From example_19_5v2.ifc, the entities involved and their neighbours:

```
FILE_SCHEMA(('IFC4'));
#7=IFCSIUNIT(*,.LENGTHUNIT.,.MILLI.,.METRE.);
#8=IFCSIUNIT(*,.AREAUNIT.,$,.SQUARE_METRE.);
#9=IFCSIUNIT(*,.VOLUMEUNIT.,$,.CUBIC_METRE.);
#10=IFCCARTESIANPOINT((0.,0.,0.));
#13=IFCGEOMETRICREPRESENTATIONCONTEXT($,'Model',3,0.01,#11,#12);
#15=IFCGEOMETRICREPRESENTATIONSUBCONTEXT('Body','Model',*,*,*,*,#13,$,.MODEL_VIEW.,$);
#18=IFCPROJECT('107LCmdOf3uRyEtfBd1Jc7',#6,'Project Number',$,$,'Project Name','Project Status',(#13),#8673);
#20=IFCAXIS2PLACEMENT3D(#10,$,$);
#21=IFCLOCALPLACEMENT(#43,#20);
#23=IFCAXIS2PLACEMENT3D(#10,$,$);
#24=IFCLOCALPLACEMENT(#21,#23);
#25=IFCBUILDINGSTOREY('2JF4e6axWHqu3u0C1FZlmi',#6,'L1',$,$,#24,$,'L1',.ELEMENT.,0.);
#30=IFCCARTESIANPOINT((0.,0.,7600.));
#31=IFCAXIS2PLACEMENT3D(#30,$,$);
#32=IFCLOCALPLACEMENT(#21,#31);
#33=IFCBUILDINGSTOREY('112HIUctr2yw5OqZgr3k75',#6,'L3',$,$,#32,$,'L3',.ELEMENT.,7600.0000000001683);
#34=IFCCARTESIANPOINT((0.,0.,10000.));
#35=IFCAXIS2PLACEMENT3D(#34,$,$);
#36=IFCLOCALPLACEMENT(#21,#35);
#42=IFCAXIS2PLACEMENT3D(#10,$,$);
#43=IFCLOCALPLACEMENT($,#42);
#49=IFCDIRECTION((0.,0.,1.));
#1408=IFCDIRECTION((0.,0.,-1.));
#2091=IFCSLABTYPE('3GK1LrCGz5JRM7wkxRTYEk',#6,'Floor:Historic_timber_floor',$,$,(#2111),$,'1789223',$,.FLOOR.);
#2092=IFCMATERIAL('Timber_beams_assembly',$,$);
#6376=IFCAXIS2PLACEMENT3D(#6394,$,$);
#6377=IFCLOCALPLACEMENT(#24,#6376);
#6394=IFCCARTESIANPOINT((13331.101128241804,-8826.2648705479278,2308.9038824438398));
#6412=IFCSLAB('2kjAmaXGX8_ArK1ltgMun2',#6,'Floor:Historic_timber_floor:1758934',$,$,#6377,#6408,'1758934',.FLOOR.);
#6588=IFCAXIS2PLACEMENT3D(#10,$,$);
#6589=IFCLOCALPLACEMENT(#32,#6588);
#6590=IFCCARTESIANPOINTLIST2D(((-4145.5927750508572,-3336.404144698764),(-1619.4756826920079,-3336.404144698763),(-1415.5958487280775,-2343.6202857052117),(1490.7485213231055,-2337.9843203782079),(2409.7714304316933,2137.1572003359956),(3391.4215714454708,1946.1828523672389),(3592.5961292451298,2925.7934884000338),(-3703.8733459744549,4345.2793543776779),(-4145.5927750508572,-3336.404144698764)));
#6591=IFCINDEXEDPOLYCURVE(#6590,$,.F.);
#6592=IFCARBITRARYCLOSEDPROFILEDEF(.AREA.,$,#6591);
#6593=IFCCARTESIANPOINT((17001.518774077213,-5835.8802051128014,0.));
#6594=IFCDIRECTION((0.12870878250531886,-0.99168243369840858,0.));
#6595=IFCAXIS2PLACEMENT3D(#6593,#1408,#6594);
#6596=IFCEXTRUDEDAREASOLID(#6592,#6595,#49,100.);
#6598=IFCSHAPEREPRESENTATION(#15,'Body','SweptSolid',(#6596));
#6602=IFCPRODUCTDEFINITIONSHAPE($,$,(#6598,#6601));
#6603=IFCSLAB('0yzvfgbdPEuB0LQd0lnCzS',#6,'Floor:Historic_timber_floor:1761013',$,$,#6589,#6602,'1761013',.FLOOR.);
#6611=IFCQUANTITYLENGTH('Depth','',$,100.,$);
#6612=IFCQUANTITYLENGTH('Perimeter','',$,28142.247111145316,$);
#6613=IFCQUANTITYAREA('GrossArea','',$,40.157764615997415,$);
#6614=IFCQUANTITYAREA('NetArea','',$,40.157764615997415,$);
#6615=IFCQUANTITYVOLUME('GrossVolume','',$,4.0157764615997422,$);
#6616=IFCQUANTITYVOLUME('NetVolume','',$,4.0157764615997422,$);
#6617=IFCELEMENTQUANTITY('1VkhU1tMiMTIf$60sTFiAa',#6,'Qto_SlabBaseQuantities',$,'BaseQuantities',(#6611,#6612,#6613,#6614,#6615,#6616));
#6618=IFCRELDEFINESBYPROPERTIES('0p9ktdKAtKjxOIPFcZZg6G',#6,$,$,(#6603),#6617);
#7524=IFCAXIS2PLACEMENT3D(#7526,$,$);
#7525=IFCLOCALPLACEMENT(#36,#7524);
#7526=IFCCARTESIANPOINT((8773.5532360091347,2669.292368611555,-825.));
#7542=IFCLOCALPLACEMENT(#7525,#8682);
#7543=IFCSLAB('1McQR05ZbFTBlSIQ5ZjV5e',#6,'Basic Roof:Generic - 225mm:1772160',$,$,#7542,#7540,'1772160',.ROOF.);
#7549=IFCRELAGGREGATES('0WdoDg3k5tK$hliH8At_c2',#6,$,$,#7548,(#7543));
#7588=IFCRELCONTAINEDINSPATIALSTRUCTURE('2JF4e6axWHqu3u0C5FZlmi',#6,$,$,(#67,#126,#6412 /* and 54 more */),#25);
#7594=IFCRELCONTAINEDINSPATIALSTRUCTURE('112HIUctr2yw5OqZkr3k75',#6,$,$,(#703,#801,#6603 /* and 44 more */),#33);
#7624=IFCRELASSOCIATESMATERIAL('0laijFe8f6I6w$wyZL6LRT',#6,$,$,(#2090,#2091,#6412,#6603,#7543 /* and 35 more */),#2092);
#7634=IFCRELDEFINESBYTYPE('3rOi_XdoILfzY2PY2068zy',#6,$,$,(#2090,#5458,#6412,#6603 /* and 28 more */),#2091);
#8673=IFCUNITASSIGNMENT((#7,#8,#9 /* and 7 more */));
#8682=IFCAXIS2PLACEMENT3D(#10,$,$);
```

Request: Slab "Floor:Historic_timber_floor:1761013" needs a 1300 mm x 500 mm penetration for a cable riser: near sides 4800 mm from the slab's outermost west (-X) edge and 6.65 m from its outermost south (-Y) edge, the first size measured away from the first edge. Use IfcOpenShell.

```python
import numpy as np
import ifcopenshell
import ifcopenshell.api.feature
import ifcopenshell.api.geometry
import ifcopenshell.api.pset
import ifcopenshell.api.root
import ifcopenshell.geom
import ifcopenshell.util.element
import ifcopenshell.util.placement
import ifcopenshell.util.representation
import ifcopenshell.util.shape
import ifcopenshell.util.unit

model = ifcopenshell.open("example_19_5v2.ifc")
unit_scale = ifcopenshell.util.unit.calculate_unit_scale(model)
area_scale = ifcopenshell.util.unit.calculate_unit_scale(model, "AREAUNIT")
volume_scale = ifcopenshell.util.unit.calculate_unit_scale(model, "VOLUMEUNIT")
settings = ifcopenshell.geom.settings()


def volume(element):
    """Net volume in cubic metres, openings subtracted."""
    shape = ifcopenshell.geom.create_shape(settings, element)
    return ifcopenshell.util.shape.get_volume(shape.geometry)


slab = model.by_guid("0yzvfgbdPEuB0LQd0lnCzS")
before = volume(slab)

# Extent in the slab's own axes, in metres. The edges named are its -X and -Y sides.
slab_shape = ifcopenshell.geom.create_shape(settings, slab)
vertices = ifcopenshell.util.shape.get_vertices(slab_shape.geometry)
x_min, y_min, bottom = vertices.min(axis=0)
top = vertices[:, 2].max()

opening = ifcopenshell.api.root.create_entity(model, ifc_class="IfcOpeningElement", name="Cable riser opening", predefined_type="OPENING")
context = ifcopenshell.util.representation.get_context(model, "Model", "Body", "MODEL_VIEW")
width, depth = 1.3, 0.5
outline = [(0.0, 0.0), (width, 0.0), (width, depth), (0.0, depth), (0.0, 0.0)]
# Overshoot both faces by 50 mm so the cut is clean.
shape = ifcopenshell.api.geometry.add_slab_representation(
    model, context=context, depth=top - bottom + 0.1, polyline=outline
)
ifcopenshell.api.geometry.assign_representation(model, product=opening, representation=shape)

matrix = ifcopenshell.util.placement.get_local_placement(slab.ObjectPlacement)
matrix[:, 3] = matrix @ np.append(np.array([x_min + 4.8, y_min + 6.65, bottom - 0.05]) / unit_scale, 1.0)
ifcopenshell.api.geometry.edit_object_placement(model, product=opening, matrix=matrix, is_si=False)
ifcopenshell.api.feature.add_feature(model, feature=opening, element=slab)

after = volume(slab)

# Update the slab's stored quantities.
qto = model.by_id(ifcopenshell.util.element.get_pset(slab, "Qto_SlabBaseQuantities", should_inherit=False)["id"])
ifcopenshell.api.pset.edit_qto(model, qto=qto, properties={
    "NetArea": after / (top - bottom) / area_scale,
    "NetVolume": after / volume_scale,
})

print(f"slab volume {before:.3f} -> {after:.3f} m3")

model.write("example_19_5v2_v2.ifc")
```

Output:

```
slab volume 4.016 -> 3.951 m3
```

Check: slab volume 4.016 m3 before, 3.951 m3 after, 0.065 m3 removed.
